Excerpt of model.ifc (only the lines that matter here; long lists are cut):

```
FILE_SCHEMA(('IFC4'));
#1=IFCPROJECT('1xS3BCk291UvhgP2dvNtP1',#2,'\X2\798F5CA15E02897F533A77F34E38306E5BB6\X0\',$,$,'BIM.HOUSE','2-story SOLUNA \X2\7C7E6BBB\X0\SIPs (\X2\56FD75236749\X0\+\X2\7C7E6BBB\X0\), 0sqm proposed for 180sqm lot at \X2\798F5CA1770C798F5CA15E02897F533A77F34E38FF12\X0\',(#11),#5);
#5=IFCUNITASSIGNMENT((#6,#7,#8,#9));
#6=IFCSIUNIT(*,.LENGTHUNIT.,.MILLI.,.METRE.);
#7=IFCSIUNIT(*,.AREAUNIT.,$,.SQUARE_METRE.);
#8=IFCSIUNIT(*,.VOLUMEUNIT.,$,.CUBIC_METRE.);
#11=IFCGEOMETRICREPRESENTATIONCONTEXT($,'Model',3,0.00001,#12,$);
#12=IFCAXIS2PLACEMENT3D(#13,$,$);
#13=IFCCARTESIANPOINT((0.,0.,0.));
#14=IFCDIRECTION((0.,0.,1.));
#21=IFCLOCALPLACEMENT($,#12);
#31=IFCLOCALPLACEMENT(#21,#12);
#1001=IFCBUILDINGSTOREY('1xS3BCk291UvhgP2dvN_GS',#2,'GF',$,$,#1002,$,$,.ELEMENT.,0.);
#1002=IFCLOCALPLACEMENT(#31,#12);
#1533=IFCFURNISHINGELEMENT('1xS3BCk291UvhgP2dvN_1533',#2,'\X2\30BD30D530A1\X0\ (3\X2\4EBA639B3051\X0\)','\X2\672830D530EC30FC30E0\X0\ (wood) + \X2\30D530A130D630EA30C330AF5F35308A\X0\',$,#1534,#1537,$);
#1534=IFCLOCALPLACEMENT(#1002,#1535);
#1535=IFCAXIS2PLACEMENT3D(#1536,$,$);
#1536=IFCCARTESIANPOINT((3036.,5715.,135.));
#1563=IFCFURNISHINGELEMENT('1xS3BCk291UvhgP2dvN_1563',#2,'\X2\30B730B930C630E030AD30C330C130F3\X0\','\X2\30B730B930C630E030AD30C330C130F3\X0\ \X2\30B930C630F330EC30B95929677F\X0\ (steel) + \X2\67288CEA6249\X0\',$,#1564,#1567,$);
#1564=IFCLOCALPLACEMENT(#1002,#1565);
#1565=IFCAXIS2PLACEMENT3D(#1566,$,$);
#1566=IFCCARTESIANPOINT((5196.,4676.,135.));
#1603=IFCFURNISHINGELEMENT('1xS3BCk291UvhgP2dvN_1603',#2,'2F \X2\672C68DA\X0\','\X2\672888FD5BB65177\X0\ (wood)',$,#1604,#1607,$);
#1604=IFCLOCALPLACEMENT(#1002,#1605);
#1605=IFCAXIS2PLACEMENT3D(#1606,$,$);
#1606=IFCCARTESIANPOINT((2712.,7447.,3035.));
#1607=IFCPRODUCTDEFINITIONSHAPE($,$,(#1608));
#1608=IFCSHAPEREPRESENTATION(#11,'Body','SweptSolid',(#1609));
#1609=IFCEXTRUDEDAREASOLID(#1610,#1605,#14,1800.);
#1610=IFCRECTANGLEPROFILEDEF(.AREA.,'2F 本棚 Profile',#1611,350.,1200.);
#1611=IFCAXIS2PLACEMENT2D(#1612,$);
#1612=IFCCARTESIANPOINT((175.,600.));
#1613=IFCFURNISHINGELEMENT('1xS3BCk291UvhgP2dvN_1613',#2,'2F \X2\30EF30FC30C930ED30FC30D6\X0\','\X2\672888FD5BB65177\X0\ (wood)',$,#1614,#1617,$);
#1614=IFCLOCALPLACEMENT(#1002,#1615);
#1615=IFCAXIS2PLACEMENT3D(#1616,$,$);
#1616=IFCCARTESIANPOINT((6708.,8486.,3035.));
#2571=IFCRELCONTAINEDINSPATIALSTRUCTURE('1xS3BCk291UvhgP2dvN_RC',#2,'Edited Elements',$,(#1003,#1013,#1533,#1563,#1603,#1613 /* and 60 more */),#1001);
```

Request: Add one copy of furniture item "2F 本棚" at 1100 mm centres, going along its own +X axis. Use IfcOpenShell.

```python
import ifcopenshell
import ifcopenshell.api.geometry
import ifcopenshell.api.root
import ifcopenshell.util.element
import ifcopenshell.util.placement

model = ifcopenshell.open("model.ifc")


def reuse_history(source, copy):
    """copy_class also copies each property set's owner history, people and application; keep the originals."""
    for rel in copy.IsDefinedBy:
        if rel.is_a("IfcRelDefinesByProperties") and (history := rel.RelatingPropertyDefinition.OwnerHistory):
            rel.RelatingPropertyDefinition.OwnerHistory = source.OwnerHistory
            ifcopenshell.util.element.remove_deep2(model, history)


source = model.by_guid("1xS3BCk291UvhgP2dvN_1603")
base = ifcopenshell.util.placement.get_local_placement(source.ObjectPlacement)
step = base[:3, 0] * 1100.0

for i in range(1, 2):
    copy = ifcopenshell.api.root.copy_class(model, product=source)
    copy.Representation = ifcopenshell.util.element.copy_deep(
        model, source.Representation, exclude=["IfcGeometricRepresentationContext", "IfcRepresentationMap"]
    )
    reuse_history(source, copy)
    matrix = base.copy()
    matrix[:3, 3] += i * step
    print("added at", matrix[:3, 3].round(3) + 0.0)
    ifcopenshell.api.geometry.edit_object_placement(model, product=copy, matrix=matrix, is_si=False)

model.write("model_edited.ifc")
```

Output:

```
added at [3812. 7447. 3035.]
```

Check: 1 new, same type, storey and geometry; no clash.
